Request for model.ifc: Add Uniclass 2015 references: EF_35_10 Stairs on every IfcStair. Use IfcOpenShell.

First a look at what the model holds.

```python
import ifcopenshell

model = ifcopenshell.open("model.ifc")
print(model.schema)
print("classifications:", [c.Name for c in model.by_type("IfcClassification")])
for ifc_class in ("IfcDoor", "IfcRoof", "IfcStair", "IfcWall", "IfcWindow"):
    print(ifc_class, len(model.by_type(ifc_class)))
```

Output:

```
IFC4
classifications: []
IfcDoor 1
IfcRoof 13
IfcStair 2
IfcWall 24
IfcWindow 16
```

```python
import ifcopenshell
import ifcopenshell.api.classification

model = ifcopenshell.open("model.ifc")

system = ifcopenshell.api.classification.add_classification(model, classification="Uniclass 2015")

codes = {
    "IfcStair": ("EF_35_10", "Stairs"),
}
for ifc_class, (code, name) in codes.items():
    products = model.by_type(ifc_class)
    ifcopenshell.api.classification.add_reference(
        model, products=products, classification=system, identification=code, name=name
    )
    print(code, len(products))

model.write("model_updated.ifc")
```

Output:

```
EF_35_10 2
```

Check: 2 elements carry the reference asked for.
